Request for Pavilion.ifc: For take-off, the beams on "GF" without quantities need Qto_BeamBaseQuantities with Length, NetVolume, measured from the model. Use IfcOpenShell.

First a look at what the model holds.

```python
import ifcopenshell
import ifcopenshell.util.element
import ifcopenshell.util.unit

model = ifcopenshell.open("Pavilion.ifc")
print(model.schema)
for unit_type in ("LENGTHUNIT", "AREAUNIT", "VOLUMEUNIT"):
    print(unit_type, ifcopenshell.util.unit.calculate_unit_scale(model, unit_type))
storey = next(s for s in model.by_type("IfcBuildingStorey") if s.Name == "GF")
beams = [e for e in ifcopenshell.util.element.get_decomposition(storey) if e.is_a("IfcBeam")]
for e in sorted(beams, key=lambda e: e.id()):
    print(e.id(), e.is_a(), e.Name, list(ifcopenshell.util.element.get_psets(e, qtos_only=True)), sep=" | ")
```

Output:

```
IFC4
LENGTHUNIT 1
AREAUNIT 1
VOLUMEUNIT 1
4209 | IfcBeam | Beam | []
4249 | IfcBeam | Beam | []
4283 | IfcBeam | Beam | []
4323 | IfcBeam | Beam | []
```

```python
import ifcopenshell
import ifcopenshell.api.pset
import ifcopenshell.geom
import ifcopenshell.util.element
import ifcopenshell.util.shape
import ifcopenshell.util.unit

model = ifcopenshell.open("Pavilion.ifc")
unit_scale = ifcopenshell.util.unit.calculate_unit_scale(model)
volume_scale = ifcopenshell.util.unit.calculate_unit_scale(model, "VOLUMEUNIT")
settings = ifcopenshell.geom.settings()

storey = next(s for s in model.by_type("IfcBuildingStorey") if s.Name == "GF")
beams = [e for e in ifcopenshell.util.element.get_decomposition(storey) if e.is_a("IfcBeam")]

for e in sorted(beams, key=lambda e: e.id()):
    if ifcopenshell.util.element.get_psets(e, qtos_only=True, should_inherit=False):
        continue
    # Geometry comes back in metres, in the element's own axes.
    shape = ifcopenshell.geom.create_shape(settings, e)
    values = {
        "Length": ifcopenshell.util.shape.get_max_xyz(shape.geometry) / unit_scale,
        "NetVolume": ifcopenshell.util.shape.get_volume(shape.geometry) / volume_scale,
    }
    qto = ifcopenshell.api.pset.add_qto(model, product=e, name="Qto_BeamBaseQuantities")
    ifcopenshell.api.pset.edit_qto(model, qto=qto, properties=values)
    print(e.id(), {k: round(v, 3) for k, v in values.items()})

model.write("Pavilion_rev.ifc")
```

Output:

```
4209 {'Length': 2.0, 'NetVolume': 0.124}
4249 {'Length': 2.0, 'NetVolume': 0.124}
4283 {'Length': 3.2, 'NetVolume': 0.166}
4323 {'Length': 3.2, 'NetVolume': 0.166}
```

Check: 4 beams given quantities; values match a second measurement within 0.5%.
